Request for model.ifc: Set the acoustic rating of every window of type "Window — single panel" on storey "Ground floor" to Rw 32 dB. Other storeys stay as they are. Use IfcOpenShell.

First a look at what the model holds.

```python
import ifcopenshell
import ifcopenshell.util.element

model = ifcopenshell.open("model.ifc")
print(model.schema)
storey = next(s for s in model.by_type("IfcBuildingStorey") if s.Name == "Ground floor")
windows = [e for e in ifcopenshell.util.element.get_decomposition(storey) if e.is_a("IfcWindow")]
seen = {}
for e in windows:
    element_type = ifcopenshell.util.element.get_type(e)
    key = (element_type.Name if element_type != e and element_type else None, ifcopenshell.util.element.get_pset(e, "Pset_WindowCommon", "AcousticRating"))
    seen[key] = seen.get(key, 0) + 1
for (name, value), count in sorted(seen.items(), key=str):
    print(count, "x", name, "|", value)
```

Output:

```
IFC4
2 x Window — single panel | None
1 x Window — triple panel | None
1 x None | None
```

```python
import ifcopenshell
import ifcopenshell.api.pset
import ifcopenshell.util.element

model = ifcopenshell.open("model.ifc")

storey = next(s for s in model.by_type("IfcBuildingStorey") if s.Name == "Ground floor")
windows = [e for e in ifcopenshell.util.element.get_decomposition(storey) if e.is_a("IfcWindow")]

count = 0
for e in windows:
    element_type = ifcopenshell.util.element.get_type(e)
    if element_type in (None, e) or element_type.Name != "Window — single panel":
        continue
    # add_pset returns the element's existing set when there is one.
    pset = ifcopenshell.api.pset.add_pset(model, product=e, name="Pset_WindowCommon")
    ifcopenshell.api.pset.edit_pset(model, pset=pset, properties={"AcousticRating": "Rw 32 dB"})
    count += 1

print(count, "windows updated")

model.write("model_rev.ifc")
```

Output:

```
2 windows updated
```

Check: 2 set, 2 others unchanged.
